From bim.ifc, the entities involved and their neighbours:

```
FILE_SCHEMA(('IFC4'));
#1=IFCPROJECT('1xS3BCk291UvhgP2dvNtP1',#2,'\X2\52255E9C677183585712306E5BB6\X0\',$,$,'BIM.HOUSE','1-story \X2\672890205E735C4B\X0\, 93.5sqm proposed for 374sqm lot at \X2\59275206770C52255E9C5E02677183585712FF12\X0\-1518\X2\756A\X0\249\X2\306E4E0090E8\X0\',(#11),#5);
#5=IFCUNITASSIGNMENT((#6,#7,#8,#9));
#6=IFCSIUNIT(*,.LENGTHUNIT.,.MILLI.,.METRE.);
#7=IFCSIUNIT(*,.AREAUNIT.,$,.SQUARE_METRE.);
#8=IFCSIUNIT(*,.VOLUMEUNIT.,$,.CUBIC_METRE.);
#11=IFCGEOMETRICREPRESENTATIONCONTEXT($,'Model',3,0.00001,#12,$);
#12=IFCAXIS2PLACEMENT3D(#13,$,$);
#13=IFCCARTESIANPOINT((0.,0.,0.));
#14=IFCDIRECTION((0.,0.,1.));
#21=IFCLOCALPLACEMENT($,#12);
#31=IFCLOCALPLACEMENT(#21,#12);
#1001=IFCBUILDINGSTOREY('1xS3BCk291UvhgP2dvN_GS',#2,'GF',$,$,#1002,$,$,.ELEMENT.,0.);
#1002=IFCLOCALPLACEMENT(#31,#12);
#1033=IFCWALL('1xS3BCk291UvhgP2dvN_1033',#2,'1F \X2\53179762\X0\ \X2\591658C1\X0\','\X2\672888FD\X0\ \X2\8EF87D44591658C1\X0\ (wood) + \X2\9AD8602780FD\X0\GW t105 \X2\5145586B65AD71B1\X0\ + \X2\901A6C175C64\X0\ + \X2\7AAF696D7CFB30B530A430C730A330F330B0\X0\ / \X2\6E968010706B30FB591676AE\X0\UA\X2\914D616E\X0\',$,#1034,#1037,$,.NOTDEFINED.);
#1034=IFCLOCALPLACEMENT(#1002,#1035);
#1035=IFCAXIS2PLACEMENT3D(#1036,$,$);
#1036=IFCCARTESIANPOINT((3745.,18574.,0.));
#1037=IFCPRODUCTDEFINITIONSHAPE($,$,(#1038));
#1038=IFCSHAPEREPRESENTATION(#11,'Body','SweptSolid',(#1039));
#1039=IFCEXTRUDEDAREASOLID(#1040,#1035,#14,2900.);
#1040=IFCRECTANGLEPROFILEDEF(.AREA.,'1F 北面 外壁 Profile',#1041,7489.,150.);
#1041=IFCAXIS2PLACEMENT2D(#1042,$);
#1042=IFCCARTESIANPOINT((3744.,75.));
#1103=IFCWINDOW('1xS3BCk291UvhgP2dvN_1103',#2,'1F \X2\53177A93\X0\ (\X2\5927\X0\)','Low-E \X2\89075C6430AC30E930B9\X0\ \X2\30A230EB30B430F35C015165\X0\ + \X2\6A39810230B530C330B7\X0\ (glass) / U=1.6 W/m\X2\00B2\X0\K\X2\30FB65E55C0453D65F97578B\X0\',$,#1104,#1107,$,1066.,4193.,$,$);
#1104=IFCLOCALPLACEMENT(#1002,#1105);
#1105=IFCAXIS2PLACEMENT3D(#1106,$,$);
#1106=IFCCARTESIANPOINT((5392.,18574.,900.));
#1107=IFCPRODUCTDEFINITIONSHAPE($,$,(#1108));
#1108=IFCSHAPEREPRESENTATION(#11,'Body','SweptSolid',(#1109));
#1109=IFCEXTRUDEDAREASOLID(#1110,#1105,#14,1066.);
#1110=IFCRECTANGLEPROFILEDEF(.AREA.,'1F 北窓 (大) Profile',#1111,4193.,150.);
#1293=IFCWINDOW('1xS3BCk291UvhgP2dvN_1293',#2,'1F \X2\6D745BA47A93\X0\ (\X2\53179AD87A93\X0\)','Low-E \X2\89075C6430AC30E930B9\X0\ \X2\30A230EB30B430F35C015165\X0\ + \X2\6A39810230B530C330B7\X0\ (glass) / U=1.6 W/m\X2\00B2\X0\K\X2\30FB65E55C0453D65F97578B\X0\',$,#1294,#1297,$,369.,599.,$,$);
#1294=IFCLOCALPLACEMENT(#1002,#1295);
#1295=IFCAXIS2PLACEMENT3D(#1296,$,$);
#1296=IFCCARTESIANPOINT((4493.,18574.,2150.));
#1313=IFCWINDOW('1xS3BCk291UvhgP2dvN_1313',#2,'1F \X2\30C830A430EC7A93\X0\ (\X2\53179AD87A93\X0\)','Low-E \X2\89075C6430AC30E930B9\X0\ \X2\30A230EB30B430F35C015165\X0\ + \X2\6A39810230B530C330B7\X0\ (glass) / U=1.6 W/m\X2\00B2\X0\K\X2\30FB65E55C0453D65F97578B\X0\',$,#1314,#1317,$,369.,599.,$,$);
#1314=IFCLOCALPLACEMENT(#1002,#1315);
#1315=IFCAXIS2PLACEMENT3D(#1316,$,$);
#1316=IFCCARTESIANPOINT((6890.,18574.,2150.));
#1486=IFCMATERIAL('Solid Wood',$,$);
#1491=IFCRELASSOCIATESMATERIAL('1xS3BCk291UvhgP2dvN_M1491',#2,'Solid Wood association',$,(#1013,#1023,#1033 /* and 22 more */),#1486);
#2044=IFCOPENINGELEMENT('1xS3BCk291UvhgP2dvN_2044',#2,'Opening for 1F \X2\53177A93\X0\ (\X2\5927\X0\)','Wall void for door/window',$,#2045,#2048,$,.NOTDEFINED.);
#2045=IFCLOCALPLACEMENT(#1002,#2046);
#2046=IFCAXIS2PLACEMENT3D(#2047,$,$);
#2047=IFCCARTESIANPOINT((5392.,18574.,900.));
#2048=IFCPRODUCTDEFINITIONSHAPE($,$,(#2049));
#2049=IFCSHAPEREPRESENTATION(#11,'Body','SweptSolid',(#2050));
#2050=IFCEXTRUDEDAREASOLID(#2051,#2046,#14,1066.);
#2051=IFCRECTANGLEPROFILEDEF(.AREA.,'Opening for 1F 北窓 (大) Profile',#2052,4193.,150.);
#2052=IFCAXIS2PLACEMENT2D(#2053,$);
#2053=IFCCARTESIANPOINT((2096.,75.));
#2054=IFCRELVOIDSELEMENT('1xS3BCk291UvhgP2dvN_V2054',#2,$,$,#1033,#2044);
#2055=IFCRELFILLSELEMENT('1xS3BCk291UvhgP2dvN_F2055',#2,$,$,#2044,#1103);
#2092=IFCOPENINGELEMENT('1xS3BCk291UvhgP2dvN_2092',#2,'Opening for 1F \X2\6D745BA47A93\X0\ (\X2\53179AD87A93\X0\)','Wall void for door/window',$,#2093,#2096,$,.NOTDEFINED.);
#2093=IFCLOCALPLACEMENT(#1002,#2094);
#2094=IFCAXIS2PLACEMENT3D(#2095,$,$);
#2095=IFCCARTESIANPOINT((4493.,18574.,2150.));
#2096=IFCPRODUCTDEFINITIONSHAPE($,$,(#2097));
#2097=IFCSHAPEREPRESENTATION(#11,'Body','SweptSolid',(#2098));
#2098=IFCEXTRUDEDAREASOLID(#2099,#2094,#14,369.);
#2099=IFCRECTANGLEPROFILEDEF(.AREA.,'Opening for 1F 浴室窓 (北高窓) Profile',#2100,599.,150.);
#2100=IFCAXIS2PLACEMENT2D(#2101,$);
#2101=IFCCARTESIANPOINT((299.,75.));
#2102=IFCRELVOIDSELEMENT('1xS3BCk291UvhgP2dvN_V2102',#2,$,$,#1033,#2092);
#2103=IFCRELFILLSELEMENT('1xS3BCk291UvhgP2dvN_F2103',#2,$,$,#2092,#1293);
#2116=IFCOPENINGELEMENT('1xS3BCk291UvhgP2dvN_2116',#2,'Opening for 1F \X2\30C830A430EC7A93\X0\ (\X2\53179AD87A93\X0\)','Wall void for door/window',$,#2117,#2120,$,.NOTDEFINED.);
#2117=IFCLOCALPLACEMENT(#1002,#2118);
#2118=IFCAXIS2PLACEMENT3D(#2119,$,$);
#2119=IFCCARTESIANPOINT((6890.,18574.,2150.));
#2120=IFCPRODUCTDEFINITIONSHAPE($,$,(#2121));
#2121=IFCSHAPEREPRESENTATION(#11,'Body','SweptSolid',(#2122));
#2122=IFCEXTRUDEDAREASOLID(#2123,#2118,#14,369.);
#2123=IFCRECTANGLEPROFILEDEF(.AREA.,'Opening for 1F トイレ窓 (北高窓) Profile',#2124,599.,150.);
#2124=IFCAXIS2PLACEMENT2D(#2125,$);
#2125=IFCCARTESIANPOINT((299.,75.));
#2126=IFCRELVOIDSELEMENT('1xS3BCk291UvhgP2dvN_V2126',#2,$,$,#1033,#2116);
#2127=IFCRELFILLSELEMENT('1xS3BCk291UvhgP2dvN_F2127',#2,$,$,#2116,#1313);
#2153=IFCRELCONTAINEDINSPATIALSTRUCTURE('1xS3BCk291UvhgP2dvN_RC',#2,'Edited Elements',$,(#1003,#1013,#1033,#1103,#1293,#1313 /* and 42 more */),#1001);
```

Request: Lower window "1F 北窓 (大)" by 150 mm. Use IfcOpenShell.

```python
import numpy as np
import ifcopenshell
import ifcopenshell.api.geometry
import ifcopenshell.util.placement
import ifcopenshell.util.unit

model = ifcopenshell.open("bim.ifc")
unit_scale = ifcopenshell.util.unit.calculate_unit_scale(model)

window = model.by_guid("1xS3BCk291UvhgP2dvN_1103")
opening = window.FillsVoids[0].RelatingOpeningElement
dz = -0.15 / unit_scale

shift = np.array([0.0, 0.0, dz])
# The window is not placed relative to its opening, so move both.
for product in (opening, window):
    matrix = ifcopenshell.util.placement.get_local_placement(product.ObjectPlacement)
    matrix[:3, 3] += shift
    ifcopenshell.api.geometry.edit_object_placement(model, product=product, matrix=matrix, is_si=False)

print(f"moved by {dz * unit_scale:+.3f} m")

model.write("bim_updated.ifc")
```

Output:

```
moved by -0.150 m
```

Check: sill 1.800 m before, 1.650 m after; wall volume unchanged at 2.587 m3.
